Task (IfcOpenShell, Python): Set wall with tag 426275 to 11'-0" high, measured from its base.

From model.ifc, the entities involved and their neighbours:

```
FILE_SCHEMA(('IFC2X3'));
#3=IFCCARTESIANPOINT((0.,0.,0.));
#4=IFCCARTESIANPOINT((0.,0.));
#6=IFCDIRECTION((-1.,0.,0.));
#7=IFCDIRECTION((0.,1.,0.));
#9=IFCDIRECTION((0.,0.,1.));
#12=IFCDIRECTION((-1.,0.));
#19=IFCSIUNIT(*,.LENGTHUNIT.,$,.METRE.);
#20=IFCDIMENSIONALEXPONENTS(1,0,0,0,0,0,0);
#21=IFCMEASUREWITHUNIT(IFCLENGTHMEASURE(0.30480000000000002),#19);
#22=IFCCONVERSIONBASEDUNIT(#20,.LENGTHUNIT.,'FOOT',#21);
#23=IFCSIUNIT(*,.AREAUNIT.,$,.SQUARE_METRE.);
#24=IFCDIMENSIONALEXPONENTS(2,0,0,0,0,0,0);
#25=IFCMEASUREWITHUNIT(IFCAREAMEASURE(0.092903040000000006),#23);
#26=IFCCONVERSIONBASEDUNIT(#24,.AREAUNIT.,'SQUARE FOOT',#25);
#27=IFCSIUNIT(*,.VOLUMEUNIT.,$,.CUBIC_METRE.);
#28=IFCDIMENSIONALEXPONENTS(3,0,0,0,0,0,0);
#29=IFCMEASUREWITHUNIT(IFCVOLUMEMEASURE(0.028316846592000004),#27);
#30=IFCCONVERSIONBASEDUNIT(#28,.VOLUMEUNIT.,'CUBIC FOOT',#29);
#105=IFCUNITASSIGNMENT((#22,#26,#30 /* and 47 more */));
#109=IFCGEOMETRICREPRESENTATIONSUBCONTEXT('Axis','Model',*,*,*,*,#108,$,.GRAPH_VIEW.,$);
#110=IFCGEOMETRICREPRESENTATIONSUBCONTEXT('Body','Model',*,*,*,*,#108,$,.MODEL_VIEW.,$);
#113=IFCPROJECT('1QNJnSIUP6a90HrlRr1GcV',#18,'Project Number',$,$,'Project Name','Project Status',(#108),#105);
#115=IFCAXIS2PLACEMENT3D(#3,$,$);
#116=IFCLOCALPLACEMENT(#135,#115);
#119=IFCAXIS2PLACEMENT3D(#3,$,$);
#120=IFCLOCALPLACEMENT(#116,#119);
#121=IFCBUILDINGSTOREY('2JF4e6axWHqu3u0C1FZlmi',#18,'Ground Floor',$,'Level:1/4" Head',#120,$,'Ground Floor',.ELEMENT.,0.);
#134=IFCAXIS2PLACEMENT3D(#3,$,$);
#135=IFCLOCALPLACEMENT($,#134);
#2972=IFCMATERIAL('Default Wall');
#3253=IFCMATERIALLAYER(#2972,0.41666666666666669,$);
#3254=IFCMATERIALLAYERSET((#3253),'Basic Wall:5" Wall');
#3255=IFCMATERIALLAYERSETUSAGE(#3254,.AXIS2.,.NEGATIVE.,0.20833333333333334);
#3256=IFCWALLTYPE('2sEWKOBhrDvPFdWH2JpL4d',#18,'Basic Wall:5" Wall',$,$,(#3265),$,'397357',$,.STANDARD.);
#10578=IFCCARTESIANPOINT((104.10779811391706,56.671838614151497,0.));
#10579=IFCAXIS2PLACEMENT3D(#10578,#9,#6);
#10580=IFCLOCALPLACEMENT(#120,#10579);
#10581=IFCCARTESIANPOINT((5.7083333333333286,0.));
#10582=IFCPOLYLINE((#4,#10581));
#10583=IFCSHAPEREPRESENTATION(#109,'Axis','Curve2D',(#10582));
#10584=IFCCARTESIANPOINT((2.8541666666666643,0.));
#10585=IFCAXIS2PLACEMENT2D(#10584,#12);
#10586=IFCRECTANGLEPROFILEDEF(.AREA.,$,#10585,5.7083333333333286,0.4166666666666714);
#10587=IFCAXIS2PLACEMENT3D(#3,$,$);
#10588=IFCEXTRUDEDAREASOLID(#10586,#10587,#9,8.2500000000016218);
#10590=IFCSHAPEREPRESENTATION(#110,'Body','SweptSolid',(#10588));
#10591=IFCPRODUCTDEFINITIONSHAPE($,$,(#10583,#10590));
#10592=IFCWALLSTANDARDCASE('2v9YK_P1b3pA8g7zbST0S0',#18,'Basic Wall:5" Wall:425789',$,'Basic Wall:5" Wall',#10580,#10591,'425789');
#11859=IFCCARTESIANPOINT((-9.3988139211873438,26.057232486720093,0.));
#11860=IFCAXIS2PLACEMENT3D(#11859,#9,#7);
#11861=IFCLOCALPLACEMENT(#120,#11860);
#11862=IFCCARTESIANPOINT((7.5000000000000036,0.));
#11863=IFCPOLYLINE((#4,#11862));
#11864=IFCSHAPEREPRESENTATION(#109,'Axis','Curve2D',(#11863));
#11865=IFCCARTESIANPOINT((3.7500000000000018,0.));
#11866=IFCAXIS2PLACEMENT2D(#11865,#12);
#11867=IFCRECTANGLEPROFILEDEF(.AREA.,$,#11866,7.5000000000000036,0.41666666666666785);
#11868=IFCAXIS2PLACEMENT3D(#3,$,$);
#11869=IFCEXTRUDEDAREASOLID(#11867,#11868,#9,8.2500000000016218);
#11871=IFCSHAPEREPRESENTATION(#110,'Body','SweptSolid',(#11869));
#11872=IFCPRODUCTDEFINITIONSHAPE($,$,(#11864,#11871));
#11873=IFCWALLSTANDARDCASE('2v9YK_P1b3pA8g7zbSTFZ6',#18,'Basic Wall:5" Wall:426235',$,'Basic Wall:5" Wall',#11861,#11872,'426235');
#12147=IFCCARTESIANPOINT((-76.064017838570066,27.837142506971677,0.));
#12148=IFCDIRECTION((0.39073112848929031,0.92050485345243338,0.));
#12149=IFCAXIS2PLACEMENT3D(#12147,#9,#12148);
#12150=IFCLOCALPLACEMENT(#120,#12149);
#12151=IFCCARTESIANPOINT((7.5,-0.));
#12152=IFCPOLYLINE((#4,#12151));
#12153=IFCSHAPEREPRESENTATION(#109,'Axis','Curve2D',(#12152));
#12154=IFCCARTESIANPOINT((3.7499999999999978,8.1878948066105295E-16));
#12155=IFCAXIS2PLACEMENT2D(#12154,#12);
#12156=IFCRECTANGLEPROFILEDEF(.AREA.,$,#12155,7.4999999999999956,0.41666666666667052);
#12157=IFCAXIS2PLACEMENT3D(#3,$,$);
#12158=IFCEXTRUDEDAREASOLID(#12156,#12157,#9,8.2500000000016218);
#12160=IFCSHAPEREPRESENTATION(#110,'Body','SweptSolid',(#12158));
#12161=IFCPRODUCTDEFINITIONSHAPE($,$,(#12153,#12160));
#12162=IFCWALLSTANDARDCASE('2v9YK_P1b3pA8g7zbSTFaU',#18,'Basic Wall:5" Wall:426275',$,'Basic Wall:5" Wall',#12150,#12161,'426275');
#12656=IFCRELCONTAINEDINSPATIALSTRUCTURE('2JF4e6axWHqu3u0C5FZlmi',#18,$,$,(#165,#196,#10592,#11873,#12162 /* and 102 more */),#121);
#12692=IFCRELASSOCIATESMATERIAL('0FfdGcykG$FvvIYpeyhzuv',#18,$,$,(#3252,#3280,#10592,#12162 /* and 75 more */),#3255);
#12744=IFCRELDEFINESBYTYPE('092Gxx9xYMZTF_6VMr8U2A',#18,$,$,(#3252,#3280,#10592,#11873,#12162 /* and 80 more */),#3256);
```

```python
import ifcopenshell
import ifcopenshell.geom
import ifcopenshell.util.representation
import ifcopenshell.util.shape
import ifcopenshell.util.unit

model = ifcopenshell.open("model.ifc")
unit_scale = ifcopenshell.util.unit.calculate_unit_scale(model)
settings = ifcopenshell.geom.settings()


def volume(element):
    """Net volume in cubic metres, openings subtracted."""
    shape = ifcopenshell.geom.create_shape(settings, element)
    return ifcopenshell.util.shape.get_volume(shape.geometry)


wall = model.by_guid("2v9YK_P1b3pA8g7zbSTFaU")
before = volume(wall)

body = ifcopenshell.util.representation.get_representation(wall, "Model", "Body")
solid = body.Items[0]
old_height = solid.Depth
solid.Depth = 132 * 0.0254 / unit_scale
after = volume(wall)

print(f"height {old_height:g} -> {solid.Depth:g}, volume {before:.3f} -> {after:.3f} m3")

model.write("model-out.ifc")
```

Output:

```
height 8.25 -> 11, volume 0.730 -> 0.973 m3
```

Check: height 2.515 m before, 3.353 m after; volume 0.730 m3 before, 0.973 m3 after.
